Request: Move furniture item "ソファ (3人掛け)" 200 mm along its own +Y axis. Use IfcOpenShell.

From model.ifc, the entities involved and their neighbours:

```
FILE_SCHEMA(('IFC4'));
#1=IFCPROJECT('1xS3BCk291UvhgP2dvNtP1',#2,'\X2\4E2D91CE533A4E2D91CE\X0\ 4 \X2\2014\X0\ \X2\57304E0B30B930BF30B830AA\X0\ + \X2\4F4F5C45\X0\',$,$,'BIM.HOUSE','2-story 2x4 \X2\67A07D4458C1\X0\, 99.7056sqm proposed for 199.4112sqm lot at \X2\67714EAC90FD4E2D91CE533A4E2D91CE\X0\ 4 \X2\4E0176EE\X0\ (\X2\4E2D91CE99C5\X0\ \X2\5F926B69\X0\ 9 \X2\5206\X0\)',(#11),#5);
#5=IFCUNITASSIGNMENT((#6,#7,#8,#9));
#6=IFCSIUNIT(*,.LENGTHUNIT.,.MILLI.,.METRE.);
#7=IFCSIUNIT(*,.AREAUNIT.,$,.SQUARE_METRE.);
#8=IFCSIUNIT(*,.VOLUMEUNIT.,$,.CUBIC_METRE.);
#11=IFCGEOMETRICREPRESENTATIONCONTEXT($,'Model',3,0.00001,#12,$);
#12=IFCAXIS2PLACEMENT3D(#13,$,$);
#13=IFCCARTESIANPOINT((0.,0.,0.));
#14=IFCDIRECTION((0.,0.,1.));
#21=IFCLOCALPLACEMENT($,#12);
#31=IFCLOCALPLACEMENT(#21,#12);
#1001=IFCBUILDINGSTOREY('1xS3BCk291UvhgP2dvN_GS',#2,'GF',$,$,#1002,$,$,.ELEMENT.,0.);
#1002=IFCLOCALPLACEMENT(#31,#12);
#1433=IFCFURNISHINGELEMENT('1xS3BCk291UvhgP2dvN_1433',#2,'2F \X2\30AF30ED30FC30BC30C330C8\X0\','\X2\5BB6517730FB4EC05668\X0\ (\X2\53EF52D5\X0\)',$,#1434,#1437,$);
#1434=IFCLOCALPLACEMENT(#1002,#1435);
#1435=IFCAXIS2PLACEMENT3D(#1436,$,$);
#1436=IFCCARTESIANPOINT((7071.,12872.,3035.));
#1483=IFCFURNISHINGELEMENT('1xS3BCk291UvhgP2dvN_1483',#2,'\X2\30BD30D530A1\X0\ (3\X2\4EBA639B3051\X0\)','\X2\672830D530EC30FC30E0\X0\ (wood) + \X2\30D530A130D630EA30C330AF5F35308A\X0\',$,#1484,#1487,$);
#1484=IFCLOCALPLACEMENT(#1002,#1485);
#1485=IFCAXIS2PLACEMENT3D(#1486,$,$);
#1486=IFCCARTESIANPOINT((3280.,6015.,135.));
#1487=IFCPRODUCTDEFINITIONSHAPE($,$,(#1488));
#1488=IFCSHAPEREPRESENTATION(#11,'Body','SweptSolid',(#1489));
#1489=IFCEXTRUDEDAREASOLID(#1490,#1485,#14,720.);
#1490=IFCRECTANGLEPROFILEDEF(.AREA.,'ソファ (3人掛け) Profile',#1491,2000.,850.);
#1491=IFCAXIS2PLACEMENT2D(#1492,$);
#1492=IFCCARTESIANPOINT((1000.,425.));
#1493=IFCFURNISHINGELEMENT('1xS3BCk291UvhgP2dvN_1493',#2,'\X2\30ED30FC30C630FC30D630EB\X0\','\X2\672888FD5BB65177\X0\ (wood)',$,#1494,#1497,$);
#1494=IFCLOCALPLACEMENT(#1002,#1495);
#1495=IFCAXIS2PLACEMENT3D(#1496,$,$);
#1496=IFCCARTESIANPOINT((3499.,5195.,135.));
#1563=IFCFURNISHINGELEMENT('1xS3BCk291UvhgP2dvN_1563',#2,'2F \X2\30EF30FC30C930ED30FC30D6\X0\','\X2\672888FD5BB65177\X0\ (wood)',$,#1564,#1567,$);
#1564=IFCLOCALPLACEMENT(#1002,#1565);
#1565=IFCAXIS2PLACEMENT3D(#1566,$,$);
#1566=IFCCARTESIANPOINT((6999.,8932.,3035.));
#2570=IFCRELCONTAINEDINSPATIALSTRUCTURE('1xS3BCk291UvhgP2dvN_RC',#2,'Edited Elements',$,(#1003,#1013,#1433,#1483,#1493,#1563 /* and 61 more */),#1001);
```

```python
import ifcopenshell
import ifcopenshell.api.geometry
import ifcopenshell.util.placement

model = ifcopenshell.open("model.ifc")

item = model.by_id(1483)
matrix = ifcopenshell.util.placement.get_local_placement(item.ObjectPlacement)
matrix[:3, 3] += matrix[:3, 1] * 200.0
ifcopenshell.api.geometry.edit_object_placement(model, product=item, matrix=matrix, is_si=False)

print(ifcopenshell.util.placement.get_local_placement(item.ObjectPlacement).round(3) + 0.0)

model.write("model-out.ifc")
```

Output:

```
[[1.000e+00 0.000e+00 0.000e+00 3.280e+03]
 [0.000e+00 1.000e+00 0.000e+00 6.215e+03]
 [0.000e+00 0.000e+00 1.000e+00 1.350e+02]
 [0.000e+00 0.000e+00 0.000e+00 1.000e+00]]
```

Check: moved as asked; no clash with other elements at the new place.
